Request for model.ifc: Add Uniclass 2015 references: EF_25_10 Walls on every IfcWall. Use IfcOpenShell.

First a look at what the model holds.

```python
import ifcopenshell

model = ifcopenshell.open("model.ifc")
print(model.schema)
print("classifications:", [c.Name for c in model.by_type("IfcClassification")])
for ifc_class in ("IfcDoor", "IfcRoof", "IfcStair", "IfcWall", "IfcWindow"):
    print(ifc_class, len(model.by_type(ifc_class)))
```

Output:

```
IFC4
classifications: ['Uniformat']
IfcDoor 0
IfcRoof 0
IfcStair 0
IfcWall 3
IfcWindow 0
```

```python
import ifcopenshell
import ifcopenshell.api.classification

model = ifcopenshell.open("model.ifc")

system = ifcopenshell.api.classification.add_classification(model, classification="Uniclass 2015")

codes = {
    "IfcWall": ("EF_25_10", "Walls"),
}
for ifc_class, (code, name) in codes.items():
    products = model.by_type(ifc_class)
    ifcopenshell.api.classification.add_reference(
        model, products=products, classification=system, identification=code, name=name
    )
    print(code, len(products))

model.write("model_edited.ifc")
```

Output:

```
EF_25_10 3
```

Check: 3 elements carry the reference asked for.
